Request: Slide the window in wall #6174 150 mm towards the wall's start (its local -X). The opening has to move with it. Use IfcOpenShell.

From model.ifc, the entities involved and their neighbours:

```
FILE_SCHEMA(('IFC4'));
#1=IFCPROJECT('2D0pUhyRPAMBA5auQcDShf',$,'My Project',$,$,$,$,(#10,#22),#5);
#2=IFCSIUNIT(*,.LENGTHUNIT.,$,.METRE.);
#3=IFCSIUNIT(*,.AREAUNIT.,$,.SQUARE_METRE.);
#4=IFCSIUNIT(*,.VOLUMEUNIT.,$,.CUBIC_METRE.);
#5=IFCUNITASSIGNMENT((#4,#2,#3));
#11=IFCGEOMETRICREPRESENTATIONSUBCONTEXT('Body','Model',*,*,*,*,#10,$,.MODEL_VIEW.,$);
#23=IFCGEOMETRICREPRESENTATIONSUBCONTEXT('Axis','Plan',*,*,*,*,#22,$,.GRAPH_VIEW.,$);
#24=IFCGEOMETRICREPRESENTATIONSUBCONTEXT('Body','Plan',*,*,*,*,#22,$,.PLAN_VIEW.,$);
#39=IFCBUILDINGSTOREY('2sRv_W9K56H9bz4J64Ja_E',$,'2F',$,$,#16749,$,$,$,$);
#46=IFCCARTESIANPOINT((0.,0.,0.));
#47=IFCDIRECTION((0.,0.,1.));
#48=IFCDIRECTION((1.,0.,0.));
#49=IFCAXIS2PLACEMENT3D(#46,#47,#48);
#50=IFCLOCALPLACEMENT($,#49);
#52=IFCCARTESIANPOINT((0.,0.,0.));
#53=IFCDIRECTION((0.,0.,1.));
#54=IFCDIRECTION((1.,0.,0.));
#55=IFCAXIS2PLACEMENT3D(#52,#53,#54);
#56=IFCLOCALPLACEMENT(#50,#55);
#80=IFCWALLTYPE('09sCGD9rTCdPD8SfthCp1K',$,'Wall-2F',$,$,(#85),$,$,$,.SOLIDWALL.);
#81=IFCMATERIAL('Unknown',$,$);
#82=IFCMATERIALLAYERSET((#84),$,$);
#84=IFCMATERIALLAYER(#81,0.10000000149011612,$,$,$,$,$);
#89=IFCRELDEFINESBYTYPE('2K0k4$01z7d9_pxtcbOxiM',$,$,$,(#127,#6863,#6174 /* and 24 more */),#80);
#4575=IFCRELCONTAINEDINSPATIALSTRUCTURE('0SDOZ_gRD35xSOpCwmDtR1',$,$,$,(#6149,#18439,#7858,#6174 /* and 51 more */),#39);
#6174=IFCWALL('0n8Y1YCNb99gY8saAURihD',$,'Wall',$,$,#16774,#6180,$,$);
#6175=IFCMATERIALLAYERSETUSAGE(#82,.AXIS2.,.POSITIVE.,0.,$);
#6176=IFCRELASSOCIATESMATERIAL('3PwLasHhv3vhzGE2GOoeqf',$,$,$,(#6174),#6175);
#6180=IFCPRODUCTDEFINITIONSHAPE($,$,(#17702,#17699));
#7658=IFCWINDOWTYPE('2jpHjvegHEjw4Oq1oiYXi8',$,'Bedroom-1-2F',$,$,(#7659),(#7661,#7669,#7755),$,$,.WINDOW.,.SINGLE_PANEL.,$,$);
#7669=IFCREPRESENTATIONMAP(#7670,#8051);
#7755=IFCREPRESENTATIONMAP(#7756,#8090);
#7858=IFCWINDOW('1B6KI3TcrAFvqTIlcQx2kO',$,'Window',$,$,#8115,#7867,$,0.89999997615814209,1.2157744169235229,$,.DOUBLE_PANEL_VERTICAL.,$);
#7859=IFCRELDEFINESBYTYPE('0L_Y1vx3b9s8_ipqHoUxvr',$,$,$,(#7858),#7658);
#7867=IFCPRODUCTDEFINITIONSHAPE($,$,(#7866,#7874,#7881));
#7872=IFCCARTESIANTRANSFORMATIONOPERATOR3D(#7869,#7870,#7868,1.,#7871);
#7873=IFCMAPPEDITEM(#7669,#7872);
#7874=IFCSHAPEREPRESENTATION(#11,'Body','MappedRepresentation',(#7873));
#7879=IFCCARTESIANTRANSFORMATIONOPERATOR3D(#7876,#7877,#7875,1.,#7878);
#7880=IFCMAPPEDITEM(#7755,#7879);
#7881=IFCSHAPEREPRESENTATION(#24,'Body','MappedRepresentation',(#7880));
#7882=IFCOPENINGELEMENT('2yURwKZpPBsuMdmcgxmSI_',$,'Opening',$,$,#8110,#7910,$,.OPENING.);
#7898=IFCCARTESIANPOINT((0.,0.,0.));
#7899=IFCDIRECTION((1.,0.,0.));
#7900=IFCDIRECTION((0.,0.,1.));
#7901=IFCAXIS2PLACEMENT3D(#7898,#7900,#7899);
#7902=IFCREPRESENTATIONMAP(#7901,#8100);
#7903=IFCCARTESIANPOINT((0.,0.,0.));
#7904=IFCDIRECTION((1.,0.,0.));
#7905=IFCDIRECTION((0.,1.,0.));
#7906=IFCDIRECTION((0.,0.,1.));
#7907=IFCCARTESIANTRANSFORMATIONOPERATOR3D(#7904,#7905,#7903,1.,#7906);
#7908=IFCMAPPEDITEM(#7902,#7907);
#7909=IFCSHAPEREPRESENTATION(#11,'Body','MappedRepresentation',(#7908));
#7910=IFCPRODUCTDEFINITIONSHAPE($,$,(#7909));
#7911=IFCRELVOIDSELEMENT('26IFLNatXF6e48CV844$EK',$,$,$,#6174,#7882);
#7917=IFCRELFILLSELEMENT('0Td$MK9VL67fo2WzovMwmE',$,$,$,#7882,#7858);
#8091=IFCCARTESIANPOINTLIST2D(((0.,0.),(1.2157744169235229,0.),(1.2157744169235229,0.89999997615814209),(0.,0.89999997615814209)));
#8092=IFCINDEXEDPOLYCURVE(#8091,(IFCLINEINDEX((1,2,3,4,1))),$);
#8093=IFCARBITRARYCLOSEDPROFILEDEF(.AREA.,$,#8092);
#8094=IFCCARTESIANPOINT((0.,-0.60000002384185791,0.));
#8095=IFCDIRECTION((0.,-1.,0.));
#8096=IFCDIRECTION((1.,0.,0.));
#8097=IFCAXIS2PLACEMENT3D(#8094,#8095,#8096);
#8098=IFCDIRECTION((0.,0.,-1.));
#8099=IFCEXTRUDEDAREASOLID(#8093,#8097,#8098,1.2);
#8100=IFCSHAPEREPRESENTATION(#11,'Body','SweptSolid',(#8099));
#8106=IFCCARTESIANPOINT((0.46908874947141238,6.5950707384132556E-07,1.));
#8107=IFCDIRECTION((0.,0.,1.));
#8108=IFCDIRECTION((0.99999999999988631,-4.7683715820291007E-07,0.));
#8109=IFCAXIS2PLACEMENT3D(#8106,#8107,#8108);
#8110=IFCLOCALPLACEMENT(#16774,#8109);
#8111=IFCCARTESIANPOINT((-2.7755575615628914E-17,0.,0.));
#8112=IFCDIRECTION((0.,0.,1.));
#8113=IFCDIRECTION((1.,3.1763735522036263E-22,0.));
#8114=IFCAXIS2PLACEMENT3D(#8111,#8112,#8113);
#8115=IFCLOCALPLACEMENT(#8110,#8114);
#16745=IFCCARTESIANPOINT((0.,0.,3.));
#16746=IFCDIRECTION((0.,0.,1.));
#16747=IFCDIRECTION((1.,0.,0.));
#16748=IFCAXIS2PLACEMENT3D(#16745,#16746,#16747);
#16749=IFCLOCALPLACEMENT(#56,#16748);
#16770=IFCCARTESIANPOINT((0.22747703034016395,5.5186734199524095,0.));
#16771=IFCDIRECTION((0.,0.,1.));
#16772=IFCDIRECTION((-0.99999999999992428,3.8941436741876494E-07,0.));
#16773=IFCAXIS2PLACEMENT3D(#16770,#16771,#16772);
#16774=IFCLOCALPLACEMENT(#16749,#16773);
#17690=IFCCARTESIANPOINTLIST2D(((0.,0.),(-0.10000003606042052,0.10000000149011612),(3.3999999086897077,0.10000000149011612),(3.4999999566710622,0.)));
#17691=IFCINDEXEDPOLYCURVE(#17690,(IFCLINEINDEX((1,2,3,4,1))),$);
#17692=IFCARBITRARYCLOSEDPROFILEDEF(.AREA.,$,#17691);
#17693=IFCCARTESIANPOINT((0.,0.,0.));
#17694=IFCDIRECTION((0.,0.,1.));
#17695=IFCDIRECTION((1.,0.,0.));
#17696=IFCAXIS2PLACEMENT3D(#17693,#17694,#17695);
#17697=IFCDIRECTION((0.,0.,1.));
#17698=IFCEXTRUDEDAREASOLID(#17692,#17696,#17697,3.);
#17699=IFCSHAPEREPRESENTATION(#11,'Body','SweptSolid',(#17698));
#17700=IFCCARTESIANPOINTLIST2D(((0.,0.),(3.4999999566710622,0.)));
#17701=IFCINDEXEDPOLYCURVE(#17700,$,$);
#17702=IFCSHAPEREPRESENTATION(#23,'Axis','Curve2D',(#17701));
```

```python
import ifcopenshell
import ifcopenshell.api.geometry
import ifcopenshell.util.placement
import ifcopenshell.util.unit

model = ifcopenshell.open("model.ifc")
unit_scale = ifcopenshell.util.unit.calculate_unit_scale(model)

window = model.by_guid("1B6KI3TcrAFvqTIlcQx2kO")
opening = window.FillsVoids[0].RelatingOpeningElement
wall = opening.VoidsElements[0].RelatingBuildingElement

wall_matrix = ifcopenshell.util.placement.get_local_placement(wall.ObjectPlacement)
shift = wall_matrix[:3, 0] * -0.15 / unit_scale
before = ifcopenshell.util.placement.get_local_placement(window.ObjectPlacement)[:3, 3].copy()

# The window is placed relative to its opening, so it follows when the opening moves.
matrix = ifcopenshell.util.placement.get_local_placement(opening.ObjectPlacement)
matrix[:3, 3] += shift
ifcopenshell.api.geometry.edit_object_placement(
    model, product=opening, matrix=matrix, is_si=False, should_transform_children=True
)

after = ifcopenshell.util.placement.get_local_placement(window.ObjectPlacement)[:3, 3]
print("window moved by", (after - before).round(3) + 0.0)

model.write("model-out.ifc")
```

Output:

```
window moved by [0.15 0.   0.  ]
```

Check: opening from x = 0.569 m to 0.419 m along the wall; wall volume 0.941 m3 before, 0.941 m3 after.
